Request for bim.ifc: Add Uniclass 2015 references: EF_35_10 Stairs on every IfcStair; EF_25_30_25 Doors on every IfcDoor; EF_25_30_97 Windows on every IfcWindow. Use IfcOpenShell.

First a look at what the model holds.

```python
import ifcopenshell

model = ifcopenshell.open("bim.ifc")
print(model.schema)
print("classifications:", [c.Name for c in model.by_type("IfcClassification")])
for ifc_class in ("IfcDoor", "IfcRoof", "IfcStair", "IfcWall", "IfcWindow"):
    print(ifc_class, len(model.by_type(ifc_class)))
```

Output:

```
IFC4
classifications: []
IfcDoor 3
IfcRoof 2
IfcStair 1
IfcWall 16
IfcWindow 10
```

```python
import ifcopenshell
import ifcopenshell.api.classification

model = ifcopenshell.open("bim.ifc")

system = ifcopenshell.api.classification.add_classification(model, classification="Uniclass 2015")

codes = {
    "IfcStair": ("EF_35_10", "Stairs"),
    "IfcDoor": ("EF_25_30_25", "Doors"),
    "IfcWindow": ("EF_25_30_97", "Windows"),
}
for ifc_class, (code, name) in codes.items():
    products = model.by_type(ifc_class)
    ifcopenshell.api.classification.add_reference(
        model, products=products, classification=system, identification=code, name=name
    )
    print(code, len(products))

model.write("bim_updated.ifc")
```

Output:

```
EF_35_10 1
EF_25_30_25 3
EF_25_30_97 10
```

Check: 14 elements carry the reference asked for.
